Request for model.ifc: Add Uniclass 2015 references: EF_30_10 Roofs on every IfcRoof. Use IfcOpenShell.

First a look at what the model holds.

```python
import ifcopenshell

model = ifcopenshell.open("model.ifc")
print(model.schema)
print("classifications:", [c.Name for c in model.by_type("IfcClassification")])
for ifc_class in ("IfcDoor", "IfcRoof", "IfcStair", "IfcWall", "IfcWindow"):
    print(ifc_class, len(model.by_type(ifc_class)))
```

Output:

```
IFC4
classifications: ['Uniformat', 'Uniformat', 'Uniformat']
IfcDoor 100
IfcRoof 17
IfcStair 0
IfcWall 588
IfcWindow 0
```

```python
import ifcopenshell
import ifcopenshell.api.classification

model = ifcopenshell.open("model.ifc")

system = ifcopenshell.api.classification.add_classification(model, classification="Uniclass 2015")

codes = {
    "IfcRoof": ("EF_30_10", "Roofs"),
}
for ifc_class, (code, name) in codes.items():
    products = model.by_type(ifc_class)
    ifcopenshell.api.classification.add_reference(
        model, products=products, classification=system, identification=code, name=name
    )
    print(code, len(products))

model.write("model_updated.ifc")
```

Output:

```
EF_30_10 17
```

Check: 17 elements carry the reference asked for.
